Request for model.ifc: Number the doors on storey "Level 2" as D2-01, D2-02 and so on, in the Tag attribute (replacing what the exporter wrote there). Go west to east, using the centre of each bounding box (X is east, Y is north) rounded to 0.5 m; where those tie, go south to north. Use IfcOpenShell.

First a look at what the model holds.

```python
import ifcopenshell
import ifcopenshell.util.element
import ifcopenshell.util.placement

model = ifcopenshell.open("model.ifc")
print(model.schema)
storey = next(s for s in model.by_type("IfcBuildingStorey") if s.Name == "Level 2")
doors = [e for e in ifcopenshell.util.element.get_decomposition(storey) if e.is_a("IfcDoor")]
for e in sorted(doors, key=lambda e: e.id()):
    origin = ifcopenshell.util.placement.get_local_placement(e.ObjectPlacement)[:3, 3]
    print(e.id(), e.Tag, e.Name, origin.round(2) + 0.0, sep=" | ")
```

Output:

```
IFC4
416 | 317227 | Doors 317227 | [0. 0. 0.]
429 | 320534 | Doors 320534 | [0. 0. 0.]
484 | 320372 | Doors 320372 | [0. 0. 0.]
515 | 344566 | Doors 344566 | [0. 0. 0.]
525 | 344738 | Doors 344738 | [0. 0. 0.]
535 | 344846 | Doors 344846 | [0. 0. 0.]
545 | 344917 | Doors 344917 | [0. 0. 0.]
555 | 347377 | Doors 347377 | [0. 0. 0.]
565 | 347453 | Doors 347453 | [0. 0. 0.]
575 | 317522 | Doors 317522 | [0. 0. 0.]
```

```python
import ifcopenshell
import ifcopenshell.geom
import ifcopenshell.util.element
import ifcopenshell.util.shape

model = ifcopenshell.open("model.ifc")
settings = ifcopenshell.geom.settings()
settings.set("use-world-coords", True)


def centre(element):
    shape = ifcopenshell.geom.create_shape(settings, element)
    return ifcopenshell.util.shape.get_bbox_centroid(shape.geometry)


storey = next(s for s in model.by_type("IfcBuildingStorey") if s.Name == "Level 2")
doors = [e for e in ifcopenshell.util.element.get_decomposition(storey) if e.is_a("IfcDoor")]

# Insertion points can sit at a corner or the storey origin, so sort by the geometry (in metres).
centres = {e: centre(e) for e in doors}
doors.sort(key=lambda e: (round(centres[e][0] / 0.5), centres[e][1]))

for i, e in enumerate(doors, start=1):
    number = f"D2-{i:02d}"
    e.Tag = number
    print(e.id(), number)

model.write("model_edited.ifc")
```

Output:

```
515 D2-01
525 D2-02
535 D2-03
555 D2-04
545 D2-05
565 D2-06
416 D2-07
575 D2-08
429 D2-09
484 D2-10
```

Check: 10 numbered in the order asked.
